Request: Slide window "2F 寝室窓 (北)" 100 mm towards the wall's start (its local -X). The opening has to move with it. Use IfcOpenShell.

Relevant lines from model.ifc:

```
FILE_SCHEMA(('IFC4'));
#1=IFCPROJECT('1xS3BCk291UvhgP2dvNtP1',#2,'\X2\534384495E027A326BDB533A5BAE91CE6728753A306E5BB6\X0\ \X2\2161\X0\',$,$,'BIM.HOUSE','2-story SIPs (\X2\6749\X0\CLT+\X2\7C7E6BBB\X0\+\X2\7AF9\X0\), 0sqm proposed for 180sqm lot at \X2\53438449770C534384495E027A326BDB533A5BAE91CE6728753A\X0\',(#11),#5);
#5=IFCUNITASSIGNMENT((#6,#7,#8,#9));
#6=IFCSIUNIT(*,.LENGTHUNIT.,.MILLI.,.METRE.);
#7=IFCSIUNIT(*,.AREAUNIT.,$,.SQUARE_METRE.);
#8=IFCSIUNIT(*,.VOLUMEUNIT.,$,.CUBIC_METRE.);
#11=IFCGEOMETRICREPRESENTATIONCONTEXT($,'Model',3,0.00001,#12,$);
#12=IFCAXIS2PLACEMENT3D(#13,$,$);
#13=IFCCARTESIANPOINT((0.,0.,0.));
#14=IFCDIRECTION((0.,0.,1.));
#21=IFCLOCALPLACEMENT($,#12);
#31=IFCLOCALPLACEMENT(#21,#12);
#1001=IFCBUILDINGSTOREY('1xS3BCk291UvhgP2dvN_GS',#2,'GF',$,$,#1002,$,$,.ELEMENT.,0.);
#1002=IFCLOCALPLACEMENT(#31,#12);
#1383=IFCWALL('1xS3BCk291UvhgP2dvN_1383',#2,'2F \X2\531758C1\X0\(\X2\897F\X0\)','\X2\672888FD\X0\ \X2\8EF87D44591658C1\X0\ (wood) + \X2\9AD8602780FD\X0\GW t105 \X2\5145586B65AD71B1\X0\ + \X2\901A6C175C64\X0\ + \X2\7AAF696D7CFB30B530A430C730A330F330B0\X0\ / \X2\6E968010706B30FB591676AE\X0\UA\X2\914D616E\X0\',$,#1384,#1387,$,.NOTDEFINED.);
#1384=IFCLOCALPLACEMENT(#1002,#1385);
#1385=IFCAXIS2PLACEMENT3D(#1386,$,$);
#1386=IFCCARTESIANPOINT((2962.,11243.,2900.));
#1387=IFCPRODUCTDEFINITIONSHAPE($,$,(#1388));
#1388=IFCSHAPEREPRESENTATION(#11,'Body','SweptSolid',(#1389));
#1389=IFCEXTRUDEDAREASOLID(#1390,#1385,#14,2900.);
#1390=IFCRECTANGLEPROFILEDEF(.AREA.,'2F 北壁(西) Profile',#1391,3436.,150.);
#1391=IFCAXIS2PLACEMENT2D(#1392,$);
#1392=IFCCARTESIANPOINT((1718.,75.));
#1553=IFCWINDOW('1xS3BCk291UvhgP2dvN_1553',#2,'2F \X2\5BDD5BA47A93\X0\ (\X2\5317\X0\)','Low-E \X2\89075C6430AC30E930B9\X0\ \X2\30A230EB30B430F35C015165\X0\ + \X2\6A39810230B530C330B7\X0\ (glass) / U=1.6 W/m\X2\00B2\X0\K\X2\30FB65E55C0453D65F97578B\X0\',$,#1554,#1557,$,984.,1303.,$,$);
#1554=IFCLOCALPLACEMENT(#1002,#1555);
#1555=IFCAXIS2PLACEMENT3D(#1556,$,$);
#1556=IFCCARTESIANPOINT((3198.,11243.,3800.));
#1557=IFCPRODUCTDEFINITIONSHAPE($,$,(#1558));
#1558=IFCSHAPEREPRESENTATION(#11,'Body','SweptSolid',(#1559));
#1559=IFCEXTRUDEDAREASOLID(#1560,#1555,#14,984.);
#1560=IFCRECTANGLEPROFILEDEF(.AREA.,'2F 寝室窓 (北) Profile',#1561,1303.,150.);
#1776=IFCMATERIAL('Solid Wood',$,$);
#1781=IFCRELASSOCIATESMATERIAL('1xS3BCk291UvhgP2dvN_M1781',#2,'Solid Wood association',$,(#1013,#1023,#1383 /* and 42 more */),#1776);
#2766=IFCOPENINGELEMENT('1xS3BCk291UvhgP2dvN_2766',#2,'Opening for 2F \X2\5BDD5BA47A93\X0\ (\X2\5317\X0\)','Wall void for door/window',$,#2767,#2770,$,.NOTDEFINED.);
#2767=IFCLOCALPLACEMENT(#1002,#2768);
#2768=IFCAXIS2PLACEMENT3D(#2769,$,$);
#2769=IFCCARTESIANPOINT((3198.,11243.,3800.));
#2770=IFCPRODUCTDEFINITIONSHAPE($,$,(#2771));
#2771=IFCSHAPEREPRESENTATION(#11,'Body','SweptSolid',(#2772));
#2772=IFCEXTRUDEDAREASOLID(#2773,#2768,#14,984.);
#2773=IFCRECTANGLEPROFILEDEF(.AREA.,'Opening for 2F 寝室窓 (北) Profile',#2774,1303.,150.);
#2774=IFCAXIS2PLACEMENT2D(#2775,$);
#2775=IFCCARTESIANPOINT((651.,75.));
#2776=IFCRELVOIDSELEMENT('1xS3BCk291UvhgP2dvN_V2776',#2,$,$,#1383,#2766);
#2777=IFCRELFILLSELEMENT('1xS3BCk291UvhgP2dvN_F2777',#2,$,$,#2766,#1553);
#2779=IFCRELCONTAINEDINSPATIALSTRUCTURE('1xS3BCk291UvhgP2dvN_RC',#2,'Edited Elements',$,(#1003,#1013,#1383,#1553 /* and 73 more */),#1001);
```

```python
import ifcopenshell
import ifcopenshell.api.geometry
import ifcopenshell.util.placement
import ifcopenshell.util.unit

model = ifcopenshell.open("model.ifc")
unit_scale = ifcopenshell.util.unit.calculate_unit_scale(model)

window = model.by_guid("1xS3BCk291UvhgP2dvN_1553")
opening = window.FillsVoids[0].RelatingOpeningElement
wall = opening.VoidsElements[0].RelatingBuildingElement

wall_matrix = ifcopenshell.util.placement.get_local_placement(wall.ObjectPlacement)
shift = wall_matrix[:3, 0] * -0.1 / unit_scale
before = ifcopenshell.util.placement.get_local_placement(window.ObjectPlacement)[:3, 3].copy()

# The window is not placed relative to its opening, so move both.
for product in (opening, window):
    matrix = ifcopenshell.util.placement.get_local_placement(product.ObjectPlacement)
    matrix[:3, 3] += shift
    ifcopenshell.api.geometry.edit_object_placement(model, product=product, matrix=matrix, is_si=False)

after = ifcopenshell.util.placement.get_local_placement(window.ObjectPlacement)[:3, 3]
print("window moved by", (after - before).round(3) + 0.0)

model.write("model_edited.ifc")
```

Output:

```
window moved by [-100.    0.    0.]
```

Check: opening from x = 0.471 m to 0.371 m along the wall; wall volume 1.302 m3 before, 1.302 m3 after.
